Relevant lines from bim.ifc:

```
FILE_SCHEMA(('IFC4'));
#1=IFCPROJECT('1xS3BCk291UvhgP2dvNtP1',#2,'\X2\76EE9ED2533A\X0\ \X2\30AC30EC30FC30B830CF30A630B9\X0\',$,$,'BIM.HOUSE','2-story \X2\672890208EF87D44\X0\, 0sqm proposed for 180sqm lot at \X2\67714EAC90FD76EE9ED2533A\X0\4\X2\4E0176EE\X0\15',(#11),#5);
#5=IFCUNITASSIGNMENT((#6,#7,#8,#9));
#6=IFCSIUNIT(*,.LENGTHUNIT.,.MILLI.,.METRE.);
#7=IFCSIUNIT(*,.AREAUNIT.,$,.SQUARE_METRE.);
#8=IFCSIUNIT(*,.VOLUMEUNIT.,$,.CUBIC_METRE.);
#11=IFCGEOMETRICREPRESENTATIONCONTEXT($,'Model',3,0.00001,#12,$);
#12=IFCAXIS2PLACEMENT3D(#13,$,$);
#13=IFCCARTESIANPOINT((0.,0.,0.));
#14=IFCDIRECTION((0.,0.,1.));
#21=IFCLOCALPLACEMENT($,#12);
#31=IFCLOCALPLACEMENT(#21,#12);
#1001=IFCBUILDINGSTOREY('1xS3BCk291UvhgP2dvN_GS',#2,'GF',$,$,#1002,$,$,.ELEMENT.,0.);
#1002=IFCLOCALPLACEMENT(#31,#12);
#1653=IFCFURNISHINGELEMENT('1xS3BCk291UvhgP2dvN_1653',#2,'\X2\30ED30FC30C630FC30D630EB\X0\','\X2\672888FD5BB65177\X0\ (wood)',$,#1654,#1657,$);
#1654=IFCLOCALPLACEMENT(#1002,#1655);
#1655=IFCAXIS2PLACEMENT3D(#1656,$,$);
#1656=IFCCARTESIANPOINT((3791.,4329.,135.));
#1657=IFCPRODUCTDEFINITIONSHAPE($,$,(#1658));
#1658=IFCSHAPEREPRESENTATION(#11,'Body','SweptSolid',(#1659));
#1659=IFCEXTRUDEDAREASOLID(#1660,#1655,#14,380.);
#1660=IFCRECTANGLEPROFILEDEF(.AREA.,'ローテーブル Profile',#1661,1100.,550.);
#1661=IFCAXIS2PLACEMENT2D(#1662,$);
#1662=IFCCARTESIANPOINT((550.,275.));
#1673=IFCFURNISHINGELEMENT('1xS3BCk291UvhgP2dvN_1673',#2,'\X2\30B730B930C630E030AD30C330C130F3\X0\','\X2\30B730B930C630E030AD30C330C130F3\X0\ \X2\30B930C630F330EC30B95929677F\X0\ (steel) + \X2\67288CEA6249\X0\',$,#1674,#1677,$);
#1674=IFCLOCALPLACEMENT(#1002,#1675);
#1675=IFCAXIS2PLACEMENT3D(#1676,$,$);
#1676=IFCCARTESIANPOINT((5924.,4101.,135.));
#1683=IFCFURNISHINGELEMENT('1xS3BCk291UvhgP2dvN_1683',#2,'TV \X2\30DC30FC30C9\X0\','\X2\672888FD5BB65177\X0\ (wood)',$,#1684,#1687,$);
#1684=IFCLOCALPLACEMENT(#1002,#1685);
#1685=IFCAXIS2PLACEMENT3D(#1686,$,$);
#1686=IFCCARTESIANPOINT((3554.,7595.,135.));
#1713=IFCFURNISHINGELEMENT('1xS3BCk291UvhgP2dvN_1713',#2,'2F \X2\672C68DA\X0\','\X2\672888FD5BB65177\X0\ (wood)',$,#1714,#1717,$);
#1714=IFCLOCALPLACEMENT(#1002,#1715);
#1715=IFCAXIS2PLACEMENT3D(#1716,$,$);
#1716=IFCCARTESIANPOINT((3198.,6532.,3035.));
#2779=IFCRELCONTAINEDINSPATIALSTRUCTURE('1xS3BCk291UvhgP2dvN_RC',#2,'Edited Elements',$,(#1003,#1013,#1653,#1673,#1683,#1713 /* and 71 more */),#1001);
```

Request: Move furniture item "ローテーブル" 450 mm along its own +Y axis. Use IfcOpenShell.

```python
import ifcopenshell
import ifcopenshell.api.geometry
import ifcopenshell.util.placement
import ifcopenshell.util.unit

model = ifcopenshell.open("bim.ifc")
unit_scale = ifcopenshell.util.unit.calculate_unit_scale(model)

item = model.by_guid("1xS3BCk291UvhgP2dvN_1653")
matrix = ifcopenshell.util.placement.get_local_placement(item.ObjectPlacement)
matrix[:3, 3] += matrix[:3, 1] * 0.45 / unit_scale
ifcopenshell.api.geometry.edit_object_placement(model, product=item, matrix=matrix, is_si=False)

print(ifcopenshell.util.placement.get_local_placement(item.ObjectPlacement).round(3) + 0.0)

model.write("bim-out.ifc")
```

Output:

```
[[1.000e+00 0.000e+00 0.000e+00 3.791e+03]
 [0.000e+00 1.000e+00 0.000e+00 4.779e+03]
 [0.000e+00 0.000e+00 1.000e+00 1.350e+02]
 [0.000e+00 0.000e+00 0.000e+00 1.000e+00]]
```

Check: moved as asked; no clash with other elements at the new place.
